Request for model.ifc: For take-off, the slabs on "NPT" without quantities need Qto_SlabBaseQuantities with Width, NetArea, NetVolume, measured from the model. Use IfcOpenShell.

First a look at what the model holds.

```python
import ifcopenshell
import ifcopenshell.util.element
import ifcopenshell.util.unit

model = ifcopenshell.open("model.ifc")
print(model.schema)
for unit_type in ("LENGTHUNIT", "AREAUNIT", "VOLUMEUNIT"):
    print(unit_type, ifcopenshell.util.unit.calculate_unit_scale(model, unit_type))
storey = next(s for s in model.by_type("IfcBuildingStorey") if s.Name == "NPT")
slabs = [e for e in ifcopenshell.util.element.get_decomposition(storey) if e.is_a("IfcSlab")]
for e in sorted(slabs, key=lambda e: e.id()):
    print(e.id(), e.is_a(), e.Name, list(ifcopenshell.util.element.get_psets(e, qtos_only=True)), sep=" | ")
```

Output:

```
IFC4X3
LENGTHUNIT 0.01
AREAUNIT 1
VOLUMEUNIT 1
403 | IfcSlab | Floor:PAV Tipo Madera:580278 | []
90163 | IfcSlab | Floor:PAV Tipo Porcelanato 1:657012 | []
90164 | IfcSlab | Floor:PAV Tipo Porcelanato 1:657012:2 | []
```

```python
import ifcopenshell
import ifcopenshell.api.pset
import ifcopenshell.geom
import ifcopenshell.util.element
import ifcopenshell.util.shape
import ifcopenshell.util.unit

model = ifcopenshell.open("model.ifc")
unit_scale = ifcopenshell.util.unit.calculate_unit_scale(model)
area_scale = ifcopenshell.util.unit.calculate_unit_scale(model, "AREAUNIT")
volume_scale = ifcopenshell.util.unit.calculate_unit_scale(model, "VOLUMEUNIT")
settings = ifcopenshell.geom.settings()

storey = next(s for s in model.by_type("IfcBuildingStorey") if s.Name == "NPT")
slabs = [e for e in ifcopenshell.util.element.get_decomposition(storey) if e.is_a("IfcSlab")]

for e in sorted(slabs, key=lambda e: e.id()):
    if ifcopenshell.util.element.get_psets(e, qtos_only=True, should_inherit=False):
        continue
    # Geometry comes back in metres, in the element's own axes.
    shape = ifcopenshell.geom.create_shape(settings, e)
    values = {
        "Width": ifcopenshell.util.shape.get_z(shape.geometry) / unit_scale,
        "NetArea": ifcopenshell.util.shape.get_footprint_area(shape.geometry) / area_scale,
        "NetVolume": ifcopenshell.util.shape.get_volume(shape.geometry) / volume_scale,
    }
    qto = ifcopenshell.api.pset.add_qto(model, product=e, name="Qto_SlabBaseQuantities")
    ifcopenshell.api.pset.edit_qto(model, qto=qto, properties=values)
    print(e.id(), {k: round(v, 3) for k, v in values.items()})

model.write("model_edited.ifc")
```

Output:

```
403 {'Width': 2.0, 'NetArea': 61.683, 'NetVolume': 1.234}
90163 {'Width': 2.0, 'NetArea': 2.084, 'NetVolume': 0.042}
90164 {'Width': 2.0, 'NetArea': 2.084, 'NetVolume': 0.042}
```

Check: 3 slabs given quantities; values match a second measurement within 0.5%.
